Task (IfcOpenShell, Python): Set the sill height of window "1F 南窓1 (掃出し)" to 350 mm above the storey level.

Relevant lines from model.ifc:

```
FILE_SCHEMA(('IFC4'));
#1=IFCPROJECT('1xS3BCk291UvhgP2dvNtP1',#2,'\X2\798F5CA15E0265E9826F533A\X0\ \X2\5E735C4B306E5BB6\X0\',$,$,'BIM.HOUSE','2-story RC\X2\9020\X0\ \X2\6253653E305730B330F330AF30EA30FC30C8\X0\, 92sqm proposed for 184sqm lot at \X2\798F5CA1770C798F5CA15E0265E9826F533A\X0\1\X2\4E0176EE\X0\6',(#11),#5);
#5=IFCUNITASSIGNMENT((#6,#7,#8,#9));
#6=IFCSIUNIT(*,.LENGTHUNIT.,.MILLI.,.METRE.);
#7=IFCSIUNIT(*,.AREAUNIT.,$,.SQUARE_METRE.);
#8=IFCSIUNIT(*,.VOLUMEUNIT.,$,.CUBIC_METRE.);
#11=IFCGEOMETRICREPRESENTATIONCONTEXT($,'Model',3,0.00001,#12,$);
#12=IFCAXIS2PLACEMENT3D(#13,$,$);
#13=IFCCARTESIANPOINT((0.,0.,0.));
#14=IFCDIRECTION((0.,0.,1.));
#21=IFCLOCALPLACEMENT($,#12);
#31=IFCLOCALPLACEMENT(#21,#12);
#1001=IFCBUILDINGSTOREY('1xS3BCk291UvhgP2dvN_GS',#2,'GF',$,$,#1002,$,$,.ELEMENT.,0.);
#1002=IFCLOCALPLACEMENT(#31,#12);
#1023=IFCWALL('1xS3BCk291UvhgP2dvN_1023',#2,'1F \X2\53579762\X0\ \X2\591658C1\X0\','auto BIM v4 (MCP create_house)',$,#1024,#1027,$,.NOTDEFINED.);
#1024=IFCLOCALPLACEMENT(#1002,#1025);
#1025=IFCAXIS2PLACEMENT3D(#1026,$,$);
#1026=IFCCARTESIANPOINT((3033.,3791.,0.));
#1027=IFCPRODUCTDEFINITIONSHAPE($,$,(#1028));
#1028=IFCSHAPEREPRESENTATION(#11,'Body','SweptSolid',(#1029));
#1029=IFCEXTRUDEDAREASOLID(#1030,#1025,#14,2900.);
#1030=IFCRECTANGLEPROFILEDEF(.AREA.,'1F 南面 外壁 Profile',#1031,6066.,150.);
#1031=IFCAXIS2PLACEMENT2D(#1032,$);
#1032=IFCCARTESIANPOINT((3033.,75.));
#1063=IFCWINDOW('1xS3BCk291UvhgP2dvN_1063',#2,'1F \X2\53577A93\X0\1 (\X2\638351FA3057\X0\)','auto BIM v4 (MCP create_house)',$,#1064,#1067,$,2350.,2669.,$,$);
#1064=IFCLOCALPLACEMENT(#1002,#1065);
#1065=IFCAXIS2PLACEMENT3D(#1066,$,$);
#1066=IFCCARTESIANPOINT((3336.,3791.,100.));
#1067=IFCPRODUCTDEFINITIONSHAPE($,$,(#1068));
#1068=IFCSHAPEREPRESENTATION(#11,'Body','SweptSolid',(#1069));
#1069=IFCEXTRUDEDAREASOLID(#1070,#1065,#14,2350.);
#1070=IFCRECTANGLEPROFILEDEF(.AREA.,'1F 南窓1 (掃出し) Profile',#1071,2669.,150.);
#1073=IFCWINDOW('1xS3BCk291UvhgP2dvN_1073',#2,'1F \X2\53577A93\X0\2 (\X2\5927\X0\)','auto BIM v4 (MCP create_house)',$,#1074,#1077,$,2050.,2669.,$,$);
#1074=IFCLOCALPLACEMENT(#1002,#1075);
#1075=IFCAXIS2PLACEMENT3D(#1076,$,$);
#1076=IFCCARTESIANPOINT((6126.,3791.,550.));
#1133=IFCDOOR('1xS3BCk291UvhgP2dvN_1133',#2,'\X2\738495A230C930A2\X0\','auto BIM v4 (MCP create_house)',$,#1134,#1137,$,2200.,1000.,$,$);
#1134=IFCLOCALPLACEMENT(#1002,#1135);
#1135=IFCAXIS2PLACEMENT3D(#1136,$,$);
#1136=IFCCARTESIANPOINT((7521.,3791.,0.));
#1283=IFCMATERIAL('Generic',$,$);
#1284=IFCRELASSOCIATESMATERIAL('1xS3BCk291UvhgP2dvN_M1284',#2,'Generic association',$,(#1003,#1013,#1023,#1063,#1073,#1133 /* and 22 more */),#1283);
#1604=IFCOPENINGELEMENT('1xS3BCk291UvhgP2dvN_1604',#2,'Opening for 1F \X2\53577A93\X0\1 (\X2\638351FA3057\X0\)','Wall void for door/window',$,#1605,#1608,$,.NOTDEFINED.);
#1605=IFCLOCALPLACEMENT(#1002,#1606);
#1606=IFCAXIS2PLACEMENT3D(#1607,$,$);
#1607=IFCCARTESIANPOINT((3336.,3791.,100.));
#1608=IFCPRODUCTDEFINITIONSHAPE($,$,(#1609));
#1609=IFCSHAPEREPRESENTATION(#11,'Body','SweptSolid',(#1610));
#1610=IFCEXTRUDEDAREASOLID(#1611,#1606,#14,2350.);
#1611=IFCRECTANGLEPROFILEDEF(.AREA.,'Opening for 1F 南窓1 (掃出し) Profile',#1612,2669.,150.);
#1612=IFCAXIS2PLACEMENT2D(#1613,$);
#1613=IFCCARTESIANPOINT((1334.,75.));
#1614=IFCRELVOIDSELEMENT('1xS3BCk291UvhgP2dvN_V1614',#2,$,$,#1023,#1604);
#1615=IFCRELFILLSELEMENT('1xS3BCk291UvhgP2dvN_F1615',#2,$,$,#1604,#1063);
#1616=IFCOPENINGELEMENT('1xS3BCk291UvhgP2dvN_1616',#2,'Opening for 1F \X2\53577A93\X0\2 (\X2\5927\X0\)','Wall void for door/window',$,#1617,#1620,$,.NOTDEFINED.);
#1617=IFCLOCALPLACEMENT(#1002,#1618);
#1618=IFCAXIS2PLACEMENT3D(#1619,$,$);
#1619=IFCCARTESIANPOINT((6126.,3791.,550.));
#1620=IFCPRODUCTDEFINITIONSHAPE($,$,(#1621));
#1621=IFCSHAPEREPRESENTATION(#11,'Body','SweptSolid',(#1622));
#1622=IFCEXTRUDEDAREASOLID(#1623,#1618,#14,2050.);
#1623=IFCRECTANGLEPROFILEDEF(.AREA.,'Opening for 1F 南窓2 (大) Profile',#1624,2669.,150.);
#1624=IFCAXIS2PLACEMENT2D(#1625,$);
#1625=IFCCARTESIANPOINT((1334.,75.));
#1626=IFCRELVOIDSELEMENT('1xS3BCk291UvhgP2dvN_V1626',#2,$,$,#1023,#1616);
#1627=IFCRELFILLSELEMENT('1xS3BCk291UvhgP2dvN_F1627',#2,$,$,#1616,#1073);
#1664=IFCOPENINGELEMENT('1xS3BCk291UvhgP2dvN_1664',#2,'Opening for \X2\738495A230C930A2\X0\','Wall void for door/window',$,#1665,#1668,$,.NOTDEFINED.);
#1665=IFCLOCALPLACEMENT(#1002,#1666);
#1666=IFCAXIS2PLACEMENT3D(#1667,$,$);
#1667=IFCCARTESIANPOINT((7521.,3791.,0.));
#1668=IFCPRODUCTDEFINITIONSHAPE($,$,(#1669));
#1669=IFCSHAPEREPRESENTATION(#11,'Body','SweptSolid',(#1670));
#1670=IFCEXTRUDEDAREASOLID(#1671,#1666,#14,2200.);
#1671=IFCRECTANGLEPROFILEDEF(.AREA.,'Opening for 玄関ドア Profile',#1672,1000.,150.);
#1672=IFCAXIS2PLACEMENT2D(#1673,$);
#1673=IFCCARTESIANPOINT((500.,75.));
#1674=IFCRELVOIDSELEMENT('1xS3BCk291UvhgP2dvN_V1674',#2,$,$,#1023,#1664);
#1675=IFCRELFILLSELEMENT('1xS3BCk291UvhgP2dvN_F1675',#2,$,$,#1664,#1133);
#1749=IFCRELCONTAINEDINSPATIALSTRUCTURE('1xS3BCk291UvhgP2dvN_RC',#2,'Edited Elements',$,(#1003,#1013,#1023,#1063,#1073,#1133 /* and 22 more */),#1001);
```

```python
import numpy as np
import ifcopenshell
import ifcopenshell.api.geometry
import ifcopenshell.geom
import ifcopenshell.util.element
import ifcopenshell.util.placement
import ifcopenshell.util.shape
import ifcopenshell.util.unit

model = ifcopenshell.open("model.ifc")
unit_scale = ifcopenshell.util.unit.calculate_unit_scale(model)

window = model.by_id(1063)
opening = window.FillsVoids[0].RelatingOpeningElement
storey = ifcopenshell.util.element.get_container(window, ifc_class="IfcBuildingStorey")
level = ifcopenshell.util.placement.get_local_placement(storey.ObjectPlacement)[2, 3]

# The opening's origin need not be at the sill, so measure its lowest point.
shape = ifcopenshell.geom.create_shape(ifcopenshell.geom.settings(), opening)
bottom = ifcopenshell.util.shape.get_shape_bottom_elevation(shape, shape.geometry) / unit_scale
dz = level + 350.0 - bottom

shift = np.array([0.0, 0.0, dz])
# The window is not placed relative to its opening, so move both.
for product in (opening, window):
    matrix = ifcopenshell.util.placement.get_local_placement(product.ObjectPlacement)
    matrix[:3, 3] += shift
    ifcopenshell.api.geometry.edit_object_placement(model, product=product, matrix=matrix, is_si=False)

print(f"moved by {dz * unit_scale:+.3f} m")

model.write("model-out.ifc")
```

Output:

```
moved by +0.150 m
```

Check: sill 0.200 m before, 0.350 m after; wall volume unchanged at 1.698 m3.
